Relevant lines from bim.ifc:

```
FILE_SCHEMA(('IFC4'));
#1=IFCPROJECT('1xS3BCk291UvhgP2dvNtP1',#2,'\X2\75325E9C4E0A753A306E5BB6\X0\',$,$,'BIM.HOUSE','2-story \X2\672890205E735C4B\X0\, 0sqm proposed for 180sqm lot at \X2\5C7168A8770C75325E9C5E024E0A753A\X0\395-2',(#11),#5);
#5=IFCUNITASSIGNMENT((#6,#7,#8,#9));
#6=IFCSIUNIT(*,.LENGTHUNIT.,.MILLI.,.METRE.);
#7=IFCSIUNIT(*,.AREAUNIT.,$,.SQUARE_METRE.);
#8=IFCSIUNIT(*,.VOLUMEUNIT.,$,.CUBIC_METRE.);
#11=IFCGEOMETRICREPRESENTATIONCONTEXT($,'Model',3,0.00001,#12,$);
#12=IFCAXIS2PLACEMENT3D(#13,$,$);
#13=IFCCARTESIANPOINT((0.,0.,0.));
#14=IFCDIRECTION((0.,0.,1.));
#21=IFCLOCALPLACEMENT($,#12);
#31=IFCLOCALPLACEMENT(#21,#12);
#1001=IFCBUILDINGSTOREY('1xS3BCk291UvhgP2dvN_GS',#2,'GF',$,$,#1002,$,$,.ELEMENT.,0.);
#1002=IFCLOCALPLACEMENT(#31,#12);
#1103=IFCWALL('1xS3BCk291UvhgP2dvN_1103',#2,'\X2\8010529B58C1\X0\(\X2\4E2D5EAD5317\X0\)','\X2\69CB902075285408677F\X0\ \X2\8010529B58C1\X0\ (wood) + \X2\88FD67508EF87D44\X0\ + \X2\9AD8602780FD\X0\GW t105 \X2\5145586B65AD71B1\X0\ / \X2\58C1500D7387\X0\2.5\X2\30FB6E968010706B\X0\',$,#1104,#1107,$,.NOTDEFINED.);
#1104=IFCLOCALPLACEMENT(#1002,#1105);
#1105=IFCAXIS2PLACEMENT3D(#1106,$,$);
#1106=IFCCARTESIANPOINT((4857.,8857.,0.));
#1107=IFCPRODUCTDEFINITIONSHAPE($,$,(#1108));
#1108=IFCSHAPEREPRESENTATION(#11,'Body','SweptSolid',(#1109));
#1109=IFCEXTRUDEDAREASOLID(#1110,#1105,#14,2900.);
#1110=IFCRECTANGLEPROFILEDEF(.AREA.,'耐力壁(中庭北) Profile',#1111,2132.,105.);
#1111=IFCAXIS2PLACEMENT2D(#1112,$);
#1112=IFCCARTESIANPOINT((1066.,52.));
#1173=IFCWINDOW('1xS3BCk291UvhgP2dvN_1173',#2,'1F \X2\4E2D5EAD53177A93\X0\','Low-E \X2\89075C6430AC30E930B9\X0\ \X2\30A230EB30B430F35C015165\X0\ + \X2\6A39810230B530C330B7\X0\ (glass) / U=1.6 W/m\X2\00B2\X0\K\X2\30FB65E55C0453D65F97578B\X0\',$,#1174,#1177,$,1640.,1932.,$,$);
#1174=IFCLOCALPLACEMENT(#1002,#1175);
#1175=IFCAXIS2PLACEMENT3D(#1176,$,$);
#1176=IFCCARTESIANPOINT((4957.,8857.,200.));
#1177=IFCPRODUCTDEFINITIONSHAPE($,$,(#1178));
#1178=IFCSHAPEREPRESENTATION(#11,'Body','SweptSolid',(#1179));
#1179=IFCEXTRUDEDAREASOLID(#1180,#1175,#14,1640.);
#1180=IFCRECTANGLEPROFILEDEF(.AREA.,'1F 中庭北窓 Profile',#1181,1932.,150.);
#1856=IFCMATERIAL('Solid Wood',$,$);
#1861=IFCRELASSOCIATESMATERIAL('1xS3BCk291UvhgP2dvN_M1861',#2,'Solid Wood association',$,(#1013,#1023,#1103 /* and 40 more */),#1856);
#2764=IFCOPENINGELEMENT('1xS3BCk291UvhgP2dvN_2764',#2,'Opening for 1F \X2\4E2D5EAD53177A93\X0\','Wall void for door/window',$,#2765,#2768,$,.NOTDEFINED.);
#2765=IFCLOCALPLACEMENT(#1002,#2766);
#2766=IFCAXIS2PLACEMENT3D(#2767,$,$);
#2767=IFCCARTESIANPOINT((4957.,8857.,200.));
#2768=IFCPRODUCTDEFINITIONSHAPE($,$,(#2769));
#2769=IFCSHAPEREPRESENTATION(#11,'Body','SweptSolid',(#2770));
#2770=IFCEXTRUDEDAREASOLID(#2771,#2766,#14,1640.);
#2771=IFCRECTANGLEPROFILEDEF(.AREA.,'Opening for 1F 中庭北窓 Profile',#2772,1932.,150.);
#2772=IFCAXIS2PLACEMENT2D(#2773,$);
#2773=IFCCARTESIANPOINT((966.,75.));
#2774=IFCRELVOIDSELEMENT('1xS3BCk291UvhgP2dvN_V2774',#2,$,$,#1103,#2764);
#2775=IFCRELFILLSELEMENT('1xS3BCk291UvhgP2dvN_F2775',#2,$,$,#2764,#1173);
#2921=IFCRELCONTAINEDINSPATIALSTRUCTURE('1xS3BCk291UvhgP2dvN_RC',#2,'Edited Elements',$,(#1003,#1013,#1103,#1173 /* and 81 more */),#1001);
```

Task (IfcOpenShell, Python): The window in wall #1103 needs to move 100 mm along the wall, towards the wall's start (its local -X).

```python
import ifcopenshell
import ifcopenshell.api.geometry
import ifcopenshell.util.placement
import ifcopenshell.util.unit

model = ifcopenshell.open("bim.ifc")
unit_scale = ifcopenshell.util.unit.calculate_unit_scale(model)

window = model.by_id(1173)
opening = window.FillsVoids[0].RelatingOpeningElement
wall = opening.VoidsElements[0].RelatingBuildingElement

wall_matrix = ifcopenshell.util.placement.get_local_placement(wall.ObjectPlacement)
shift = wall_matrix[:3, 0] * -0.1 / unit_scale
before = ifcopenshell.util.placement.get_local_placement(window.ObjectPlacement)[:3, 3].copy()

# The window is not placed relative to its opening, so move both.
for product in (opening, window):
    matrix = ifcopenshell.util.placement.get_local_placement(product.ObjectPlacement)
    matrix[:3, 3] += shift
    ifcopenshell.api.geometry.edit_object_placement(model, product=product, matrix=matrix, is_si=False)

after = ifcopenshell.util.placement.get_local_placement(window.ObjectPlacement)[:3, 3]
print("window moved by", (after - before).round(3) + 0.0)

model.write("bim_edited.ifc")
```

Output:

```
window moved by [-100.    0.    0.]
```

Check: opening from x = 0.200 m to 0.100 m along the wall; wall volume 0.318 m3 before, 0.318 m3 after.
